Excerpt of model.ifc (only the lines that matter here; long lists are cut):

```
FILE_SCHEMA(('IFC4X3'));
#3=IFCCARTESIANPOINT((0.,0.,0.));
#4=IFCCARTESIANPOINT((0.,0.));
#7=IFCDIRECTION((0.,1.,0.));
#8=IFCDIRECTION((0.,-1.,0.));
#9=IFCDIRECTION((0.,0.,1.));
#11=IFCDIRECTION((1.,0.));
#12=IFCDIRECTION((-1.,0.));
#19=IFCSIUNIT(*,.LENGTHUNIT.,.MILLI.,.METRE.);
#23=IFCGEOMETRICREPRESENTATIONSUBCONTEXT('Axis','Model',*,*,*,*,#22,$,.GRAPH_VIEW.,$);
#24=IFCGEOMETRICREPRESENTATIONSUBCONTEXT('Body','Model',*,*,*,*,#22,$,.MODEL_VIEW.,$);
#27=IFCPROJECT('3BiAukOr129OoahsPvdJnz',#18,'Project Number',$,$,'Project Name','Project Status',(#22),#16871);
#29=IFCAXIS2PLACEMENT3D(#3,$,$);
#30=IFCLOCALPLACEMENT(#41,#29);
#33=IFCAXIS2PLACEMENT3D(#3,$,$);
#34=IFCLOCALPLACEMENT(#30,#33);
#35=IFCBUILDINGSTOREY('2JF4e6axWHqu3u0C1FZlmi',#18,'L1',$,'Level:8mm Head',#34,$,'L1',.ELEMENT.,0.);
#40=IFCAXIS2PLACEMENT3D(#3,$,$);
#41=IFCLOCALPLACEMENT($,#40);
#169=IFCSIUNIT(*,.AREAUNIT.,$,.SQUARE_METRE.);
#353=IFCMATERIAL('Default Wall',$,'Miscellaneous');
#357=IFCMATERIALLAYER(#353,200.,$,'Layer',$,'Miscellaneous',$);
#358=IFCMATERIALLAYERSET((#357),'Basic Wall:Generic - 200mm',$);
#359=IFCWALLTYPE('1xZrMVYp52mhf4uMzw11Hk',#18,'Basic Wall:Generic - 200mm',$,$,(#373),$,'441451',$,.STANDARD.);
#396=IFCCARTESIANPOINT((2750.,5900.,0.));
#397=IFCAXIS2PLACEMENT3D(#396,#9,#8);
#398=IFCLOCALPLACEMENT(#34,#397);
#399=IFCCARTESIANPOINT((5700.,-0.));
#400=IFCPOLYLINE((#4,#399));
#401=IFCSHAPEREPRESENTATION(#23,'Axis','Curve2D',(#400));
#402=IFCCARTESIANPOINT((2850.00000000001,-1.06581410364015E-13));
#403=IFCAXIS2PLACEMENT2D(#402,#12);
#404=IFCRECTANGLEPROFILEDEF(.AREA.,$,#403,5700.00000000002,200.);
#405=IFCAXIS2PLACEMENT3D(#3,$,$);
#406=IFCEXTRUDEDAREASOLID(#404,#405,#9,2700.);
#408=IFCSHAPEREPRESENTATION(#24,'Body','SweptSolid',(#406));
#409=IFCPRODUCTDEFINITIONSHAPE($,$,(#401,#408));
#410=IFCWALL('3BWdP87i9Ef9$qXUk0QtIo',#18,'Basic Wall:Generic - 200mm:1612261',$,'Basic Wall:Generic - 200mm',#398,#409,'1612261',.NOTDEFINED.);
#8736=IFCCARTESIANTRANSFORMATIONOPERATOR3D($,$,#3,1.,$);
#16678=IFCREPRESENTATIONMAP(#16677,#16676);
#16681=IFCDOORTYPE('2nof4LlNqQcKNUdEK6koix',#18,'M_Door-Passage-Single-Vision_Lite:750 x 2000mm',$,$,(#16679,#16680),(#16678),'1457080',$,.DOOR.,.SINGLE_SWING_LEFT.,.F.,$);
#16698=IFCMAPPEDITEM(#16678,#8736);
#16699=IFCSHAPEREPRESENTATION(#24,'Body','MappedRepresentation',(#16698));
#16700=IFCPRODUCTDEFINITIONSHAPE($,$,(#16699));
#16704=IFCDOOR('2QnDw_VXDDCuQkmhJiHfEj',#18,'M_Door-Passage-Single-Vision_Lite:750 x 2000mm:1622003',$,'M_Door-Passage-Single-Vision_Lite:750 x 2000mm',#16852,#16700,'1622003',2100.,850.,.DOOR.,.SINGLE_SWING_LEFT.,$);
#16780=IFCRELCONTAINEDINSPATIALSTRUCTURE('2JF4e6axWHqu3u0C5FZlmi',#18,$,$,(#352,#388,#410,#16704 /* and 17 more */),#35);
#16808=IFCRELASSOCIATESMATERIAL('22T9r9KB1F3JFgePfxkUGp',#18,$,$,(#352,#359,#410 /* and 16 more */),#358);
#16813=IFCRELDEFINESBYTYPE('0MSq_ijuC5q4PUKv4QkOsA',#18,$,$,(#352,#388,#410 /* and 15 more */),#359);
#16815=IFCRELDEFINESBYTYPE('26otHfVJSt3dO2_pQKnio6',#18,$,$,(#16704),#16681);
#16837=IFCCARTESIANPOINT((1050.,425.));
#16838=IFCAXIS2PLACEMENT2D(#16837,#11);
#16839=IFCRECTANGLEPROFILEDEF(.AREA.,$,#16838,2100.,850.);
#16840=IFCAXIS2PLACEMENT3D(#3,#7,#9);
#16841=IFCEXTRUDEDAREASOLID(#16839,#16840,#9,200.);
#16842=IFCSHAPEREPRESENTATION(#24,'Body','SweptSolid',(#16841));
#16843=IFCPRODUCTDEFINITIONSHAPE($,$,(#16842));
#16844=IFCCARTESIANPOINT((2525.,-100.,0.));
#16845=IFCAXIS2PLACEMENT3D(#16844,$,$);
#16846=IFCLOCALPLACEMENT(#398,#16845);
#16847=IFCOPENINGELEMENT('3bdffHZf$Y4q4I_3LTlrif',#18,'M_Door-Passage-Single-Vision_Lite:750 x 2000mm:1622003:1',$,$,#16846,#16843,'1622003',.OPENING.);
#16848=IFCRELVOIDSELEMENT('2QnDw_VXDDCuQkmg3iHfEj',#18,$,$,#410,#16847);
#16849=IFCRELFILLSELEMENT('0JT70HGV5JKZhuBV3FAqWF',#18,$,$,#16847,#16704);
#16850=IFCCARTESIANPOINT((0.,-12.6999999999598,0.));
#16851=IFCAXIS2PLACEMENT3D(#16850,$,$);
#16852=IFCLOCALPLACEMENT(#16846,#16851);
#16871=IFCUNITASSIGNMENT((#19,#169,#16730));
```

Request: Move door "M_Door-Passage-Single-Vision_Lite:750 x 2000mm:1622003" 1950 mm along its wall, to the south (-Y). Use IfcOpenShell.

```python
import ifcopenshell
import ifcopenshell.api.geometry
import ifcopenshell.util.placement
import ifcopenshell.util.unit

model = ifcopenshell.open("model.ifc")
unit_scale = ifcopenshell.util.unit.calculate_unit_scale(model)

door = model.by_guid("2QnDw_VXDDCuQkmhJiHfEj")
opening = door.FillsVoids[0].RelatingOpeningElement
wall = opening.VoidsElements[0].RelatingBuildingElement

wall_matrix = ifcopenshell.util.placement.get_local_placement(wall.ObjectPlacement)
shift = wall_matrix[:3, 0] * 1.95 / unit_scale
before = ifcopenshell.util.placement.get_local_placement(door.ObjectPlacement)[:3, 3].copy()

# The door is placed relative to its opening, so it follows when the opening moves.
matrix = ifcopenshell.util.placement.get_local_placement(opening.ObjectPlacement)
matrix[:3, 3] += shift
ifcopenshell.api.geometry.edit_object_placement(
    model, product=opening, matrix=matrix, is_si=False, should_transform_children=True
)

after = ifcopenshell.util.placement.get_local_placement(door.ObjectPlacement)[:3, 3]
print("door moved by", (after - before).round(3) + 0.0)

model.write("model_edited.ifc")
```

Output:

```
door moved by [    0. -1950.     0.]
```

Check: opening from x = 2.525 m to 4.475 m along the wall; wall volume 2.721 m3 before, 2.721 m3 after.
